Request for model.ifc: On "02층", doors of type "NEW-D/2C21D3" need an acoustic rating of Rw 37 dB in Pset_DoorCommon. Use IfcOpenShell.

First a look at what the model holds.

```python
import ifcopenshell
import ifcopenshell.util.element

model = ifcopenshell.open("model.ifc")
print(model.schema)
storey = next(s for s in model.by_type("IfcBuildingStorey") if s.Name == "02층")
doors = [e for e in ifcopenshell.util.element.get_decomposition(storey) if e.is_a("IfcDoor")]
seen = {}
for e in doors:
    element_type = ifcopenshell.util.element.get_type(e)
    key = (element_type.Name if element_type != e and element_type else None, ifcopenshell.util.element.get_pset(e, "Pset_DoorCommon", "AcousticRating"))
    seen[key] = seen.get(key, 0) + 1
for (name, value), count in sorted(seen.items(), key=str):
    print(count, "x", name, "|", value)
```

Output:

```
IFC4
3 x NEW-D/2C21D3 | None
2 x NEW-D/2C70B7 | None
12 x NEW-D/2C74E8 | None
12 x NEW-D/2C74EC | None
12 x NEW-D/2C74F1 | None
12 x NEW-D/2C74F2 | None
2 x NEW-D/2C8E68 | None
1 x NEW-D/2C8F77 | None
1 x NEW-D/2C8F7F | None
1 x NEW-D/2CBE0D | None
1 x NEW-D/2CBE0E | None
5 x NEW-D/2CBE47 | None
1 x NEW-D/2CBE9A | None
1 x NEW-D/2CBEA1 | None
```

```python
import ifcopenshell
import ifcopenshell.api.pset
import ifcopenshell.util.element

model = ifcopenshell.open("model.ifc")

storey = next(s for s in model.by_type("IfcBuildingStorey") if s.Name == "02층")
doors = [e for e in ifcopenshell.util.element.get_decomposition(storey) if e.is_a("IfcDoor")]

count = 0
for e in doors:
    element_type = ifcopenshell.util.element.get_type(e)
    if element_type in (None, e) or element_type.Name != "NEW-D/2C21D3":
        continue
    # add_pset returns the element's existing set when there is one.
    pset = ifcopenshell.api.pset.add_pset(model, product=e, name="Pset_DoorCommon")
    ifcopenshell.api.pset.edit_pset(model, pset=pset, properties={"AcousticRating": "Rw 37 dB"})
    count += 1

print(count, "doors updated")

model.write("model_edited.ifc")
```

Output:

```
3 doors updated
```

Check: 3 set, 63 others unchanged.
